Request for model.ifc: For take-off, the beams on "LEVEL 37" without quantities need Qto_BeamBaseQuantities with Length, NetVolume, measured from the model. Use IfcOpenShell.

First a look at what the model holds.

```python
import ifcopenshell
import ifcopenshell.util.element
import ifcopenshell.util.unit

model = ifcopenshell.open("model.ifc")
print(model.schema)
for unit_type in ("LENGTHUNIT", "AREAUNIT", "VOLUMEUNIT"):
    print(unit_type, ifcopenshell.util.unit.calculate_unit_scale(model, unit_type))
storey = next(s for s in model.by_type("IfcBuildingStorey") if s.Name == "LEVEL 37")
beams = [e for e in ifcopenshell.util.element.get_decomposition(storey) if e.is_a("IfcBeam")]
for e in sorted(beams, key=lambda e: e.id()):
    print(e.id(), e.is_a(), e.Name, list(ifcopenshell.util.element.get_psets(e, qtos_only=True)), sep=" | ")
```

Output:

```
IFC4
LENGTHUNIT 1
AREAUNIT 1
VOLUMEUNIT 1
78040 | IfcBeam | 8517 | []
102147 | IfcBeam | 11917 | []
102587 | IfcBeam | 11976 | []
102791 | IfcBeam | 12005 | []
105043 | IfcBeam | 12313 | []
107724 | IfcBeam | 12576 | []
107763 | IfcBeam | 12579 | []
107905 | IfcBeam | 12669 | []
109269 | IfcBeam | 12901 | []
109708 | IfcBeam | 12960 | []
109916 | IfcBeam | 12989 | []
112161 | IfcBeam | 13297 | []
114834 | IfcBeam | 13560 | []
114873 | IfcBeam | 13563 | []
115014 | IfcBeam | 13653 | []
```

```python
import ifcopenshell
import ifcopenshell.api.pset
import ifcopenshell.geom
import ifcopenshell.util.element
import ifcopenshell.util.shape
import ifcopenshell.util.unit

model = ifcopenshell.open("model.ifc")
unit_scale = ifcopenshell.util.unit.calculate_unit_scale(model)
volume_scale = ifcopenshell.util.unit.calculate_unit_scale(model, "VOLUMEUNIT")
settings = ifcopenshell.geom.settings()

storey = next(s for s in model.by_type("IfcBuildingStorey") if s.Name == "LEVEL 37")
beams = [e for e in ifcopenshell.util.element.get_decomposition(storey) if e.is_a("IfcBeam")]

for e in sorted(beams, key=lambda e: e.id()):
    if ifcopenshell.util.element.get_psets(e, qtos_only=True, should_inherit=False):
        continue
    # Geometry comes back in metres, in the element's own axes.
    shape = ifcopenshell.geom.create_shape(settings, e)
    values = {
        "Length": ifcopenshell.util.shape.get_max_xyz(shape.geometry) / unit_scale,
        "NetVolume": ifcopenshell.util.shape.get_volume(shape.geometry) / volume_scale,
    }
    qto = ifcopenshell.api.pset.add_qto(model, product=e, name="Qto_BeamBaseQuantities")
    ifcopenshell.api.pset.edit_qto(model, qto=qto, properties=values)
    print(e.id(), {k: round(v, 3) for k, v in values.items()})

model.write("model-out.ifc")
```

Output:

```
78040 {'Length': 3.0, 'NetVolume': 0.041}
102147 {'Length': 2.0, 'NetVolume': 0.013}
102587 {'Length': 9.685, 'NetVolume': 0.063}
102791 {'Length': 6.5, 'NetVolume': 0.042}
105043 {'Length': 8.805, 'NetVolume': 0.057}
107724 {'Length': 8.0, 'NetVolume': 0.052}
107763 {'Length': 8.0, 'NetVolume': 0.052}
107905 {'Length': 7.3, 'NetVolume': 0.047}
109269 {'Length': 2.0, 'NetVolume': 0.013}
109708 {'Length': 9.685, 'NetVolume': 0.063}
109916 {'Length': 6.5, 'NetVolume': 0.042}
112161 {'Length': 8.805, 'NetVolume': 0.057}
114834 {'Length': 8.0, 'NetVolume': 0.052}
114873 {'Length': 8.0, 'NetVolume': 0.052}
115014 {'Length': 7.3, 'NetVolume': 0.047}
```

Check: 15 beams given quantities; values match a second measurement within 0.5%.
